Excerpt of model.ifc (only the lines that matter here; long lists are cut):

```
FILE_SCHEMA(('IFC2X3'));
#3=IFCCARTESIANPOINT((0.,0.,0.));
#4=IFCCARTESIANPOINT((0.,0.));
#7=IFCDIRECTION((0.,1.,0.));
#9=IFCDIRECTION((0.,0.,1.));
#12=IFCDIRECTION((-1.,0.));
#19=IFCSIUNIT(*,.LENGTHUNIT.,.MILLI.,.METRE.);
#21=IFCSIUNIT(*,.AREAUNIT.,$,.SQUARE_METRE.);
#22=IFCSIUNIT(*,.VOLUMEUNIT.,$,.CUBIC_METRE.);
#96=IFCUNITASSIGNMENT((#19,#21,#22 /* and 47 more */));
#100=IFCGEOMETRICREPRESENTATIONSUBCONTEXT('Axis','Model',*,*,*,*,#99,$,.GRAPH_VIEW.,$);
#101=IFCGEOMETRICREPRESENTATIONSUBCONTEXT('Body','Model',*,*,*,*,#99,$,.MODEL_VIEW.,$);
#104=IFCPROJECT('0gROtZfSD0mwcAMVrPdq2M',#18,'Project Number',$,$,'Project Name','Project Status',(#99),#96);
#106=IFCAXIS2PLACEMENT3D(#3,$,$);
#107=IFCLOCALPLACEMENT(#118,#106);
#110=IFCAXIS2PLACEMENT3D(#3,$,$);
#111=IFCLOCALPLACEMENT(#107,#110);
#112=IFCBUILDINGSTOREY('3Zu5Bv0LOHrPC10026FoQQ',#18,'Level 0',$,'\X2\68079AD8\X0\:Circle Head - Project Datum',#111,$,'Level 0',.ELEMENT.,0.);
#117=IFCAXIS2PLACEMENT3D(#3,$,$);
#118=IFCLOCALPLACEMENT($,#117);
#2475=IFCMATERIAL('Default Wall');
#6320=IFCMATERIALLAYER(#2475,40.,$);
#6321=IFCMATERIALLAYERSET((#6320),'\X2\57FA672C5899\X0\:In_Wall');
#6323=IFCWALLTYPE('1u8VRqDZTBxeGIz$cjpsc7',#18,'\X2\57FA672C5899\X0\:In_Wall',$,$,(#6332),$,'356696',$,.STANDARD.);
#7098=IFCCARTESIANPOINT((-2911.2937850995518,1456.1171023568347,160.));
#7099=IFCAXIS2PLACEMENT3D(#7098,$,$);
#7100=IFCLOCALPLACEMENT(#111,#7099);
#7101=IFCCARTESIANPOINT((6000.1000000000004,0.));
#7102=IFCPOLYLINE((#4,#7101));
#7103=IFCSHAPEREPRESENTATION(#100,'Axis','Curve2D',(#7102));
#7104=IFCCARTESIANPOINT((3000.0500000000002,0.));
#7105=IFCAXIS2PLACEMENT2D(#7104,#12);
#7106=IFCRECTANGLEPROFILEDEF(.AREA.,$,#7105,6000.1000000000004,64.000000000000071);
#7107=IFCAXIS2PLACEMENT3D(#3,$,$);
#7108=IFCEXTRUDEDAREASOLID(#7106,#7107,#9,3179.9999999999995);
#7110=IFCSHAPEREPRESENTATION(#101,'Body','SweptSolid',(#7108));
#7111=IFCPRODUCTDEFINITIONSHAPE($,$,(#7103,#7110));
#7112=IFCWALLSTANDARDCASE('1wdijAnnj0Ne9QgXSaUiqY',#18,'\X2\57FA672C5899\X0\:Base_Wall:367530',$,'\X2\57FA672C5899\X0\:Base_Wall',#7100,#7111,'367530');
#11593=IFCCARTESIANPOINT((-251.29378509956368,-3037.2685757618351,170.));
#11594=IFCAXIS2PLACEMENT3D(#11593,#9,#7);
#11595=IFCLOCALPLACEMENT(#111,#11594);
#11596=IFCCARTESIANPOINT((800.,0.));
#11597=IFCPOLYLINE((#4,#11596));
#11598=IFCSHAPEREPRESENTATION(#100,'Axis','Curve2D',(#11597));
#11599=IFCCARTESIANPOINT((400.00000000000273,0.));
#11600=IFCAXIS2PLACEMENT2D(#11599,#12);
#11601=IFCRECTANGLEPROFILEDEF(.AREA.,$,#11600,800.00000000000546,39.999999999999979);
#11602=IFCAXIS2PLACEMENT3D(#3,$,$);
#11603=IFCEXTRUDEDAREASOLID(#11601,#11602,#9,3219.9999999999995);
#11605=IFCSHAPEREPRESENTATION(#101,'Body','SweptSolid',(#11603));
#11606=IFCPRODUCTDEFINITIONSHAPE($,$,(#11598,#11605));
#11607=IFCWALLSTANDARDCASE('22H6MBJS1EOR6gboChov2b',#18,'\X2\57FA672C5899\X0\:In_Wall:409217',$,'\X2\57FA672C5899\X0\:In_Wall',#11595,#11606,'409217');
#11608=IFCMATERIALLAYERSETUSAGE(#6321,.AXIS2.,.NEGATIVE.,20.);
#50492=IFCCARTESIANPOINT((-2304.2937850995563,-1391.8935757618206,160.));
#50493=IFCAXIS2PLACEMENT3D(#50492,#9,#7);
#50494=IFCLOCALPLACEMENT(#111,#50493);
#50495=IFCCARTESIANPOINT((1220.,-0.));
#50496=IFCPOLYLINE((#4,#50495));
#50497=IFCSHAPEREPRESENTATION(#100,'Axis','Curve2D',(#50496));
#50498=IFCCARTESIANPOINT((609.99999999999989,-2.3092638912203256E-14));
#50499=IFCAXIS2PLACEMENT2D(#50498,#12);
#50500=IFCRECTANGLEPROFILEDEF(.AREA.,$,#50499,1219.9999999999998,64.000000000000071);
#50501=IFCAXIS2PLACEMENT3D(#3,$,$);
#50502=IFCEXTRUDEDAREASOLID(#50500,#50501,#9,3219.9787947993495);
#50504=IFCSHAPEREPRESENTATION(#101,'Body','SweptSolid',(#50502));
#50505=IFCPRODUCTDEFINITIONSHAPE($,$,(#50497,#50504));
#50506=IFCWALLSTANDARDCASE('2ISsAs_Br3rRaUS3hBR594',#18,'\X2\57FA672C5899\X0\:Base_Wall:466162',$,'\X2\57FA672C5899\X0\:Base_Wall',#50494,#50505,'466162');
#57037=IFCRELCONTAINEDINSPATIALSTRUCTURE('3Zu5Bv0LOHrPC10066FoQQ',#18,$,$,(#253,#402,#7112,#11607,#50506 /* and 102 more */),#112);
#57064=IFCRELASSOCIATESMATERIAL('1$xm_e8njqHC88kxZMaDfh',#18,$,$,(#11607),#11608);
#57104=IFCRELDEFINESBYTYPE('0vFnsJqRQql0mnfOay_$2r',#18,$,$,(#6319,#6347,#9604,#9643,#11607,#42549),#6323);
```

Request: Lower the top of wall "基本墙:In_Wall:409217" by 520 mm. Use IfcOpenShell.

```python
import ifcopenshell
import ifcopenshell.geom
import ifcopenshell.util.representation
import ifcopenshell.util.shape

model = ifcopenshell.open("model.ifc")
settings = ifcopenshell.geom.settings()


def volume(element):
    """Net volume in cubic metres, openings subtracted."""
    shape = ifcopenshell.geom.create_shape(settings, element)
    return ifcopenshell.util.shape.get_volume(shape.geometry)


wall = model.by_guid("22H6MBJS1EOR6gboChov2b")
before = volume(wall)

body = ifcopenshell.util.representation.get_representation(wall, "Model", "Body")
solid = body.Items[0]
old_height = solid.Depth
solid.Depth -= 520.0
after = volume(wall)

print(f"height {old_height:g} -> {solid.Depth:g}, volume {before:.3f} -> {after:.3f} m3")

model.write("model_rev.ifc")
```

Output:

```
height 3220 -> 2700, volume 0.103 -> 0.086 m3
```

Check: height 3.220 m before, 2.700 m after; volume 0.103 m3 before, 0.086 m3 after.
